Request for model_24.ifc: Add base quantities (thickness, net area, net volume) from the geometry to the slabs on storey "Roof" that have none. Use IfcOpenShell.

First a look at what the model holds.

```python
import ifcopenshell
import ifcopenshell.util.element
import ifcopenshell.util.unit

model = ifcopenshell.open("model_24.ifc")
print(model.schema)
for unit_type in ("LENGTHUNIT", "AREAUNIT", "VOLUMEUNIT"):
    print(unit_type, ifcopenshell.util.unit.calculate_unit_scale(model, unit_type))
storey = next(s for s in model.by_type("IfcBuildingStorey") if s.Name == "Roof")
slabs = [e for e in ifcopenshell.util.element.get_decomposition(storey) if e.is_a("IfcSlab")]
for e in sorted(slabs, key=lambda e: e.id()):
    print(e.id(), e.is_a(), e.Name, list(ifcopenshell.util.element.get_psets(e, qtos_only=True)), sep=" | ")
```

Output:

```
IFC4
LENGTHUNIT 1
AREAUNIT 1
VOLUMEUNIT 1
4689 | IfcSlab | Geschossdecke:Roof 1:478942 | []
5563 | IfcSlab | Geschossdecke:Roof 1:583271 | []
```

```python
import ifcopenshell
import ifcopenshell.api.pset
import ifcopenshell.geom
import ifcopenshell.util.element
import ifcopenshell.util.shape
import ifcopenshell.util.unit

model = ifcopenshell.open("model_24.ifc")
unit_scale = ifcopenshell.util.unit.calculate_unit_scale(model)
area_scale = ifcopenshell.util.unit.calculate_unit_scale(model, "AREAUNIT")
volume_scale = ifcopenshell.util.unit.calculate_unit_scale(model, "VOLUMEUNIT")
settings = ifcopenshell.geom.settings()

storey = next(s for s in model.by_type("IfcBuildingStorey") if s.Name == "Roof")
slabs = [e for e in ifcopenshell.util.element.get_decomposition(storey) if e.is_a("IfcSlab")]

for e in sorted(slabs, key=lambda e: e.id()):
    if ifcopenshell.util.element.get_psets(e, qtos_only=True, should_inherit=False):
        continue
    # Geometry comes back in metres, in the element's own axes.
    shape = ifcopenshell.geom.create_shape(settings, e)
    values = {
        "Width": ifcopenshell.util.shape.get_z(shape.geometry) / unit_scale,
        "NetArea": ifcopenshell.util.shape.get_footprint_area(shape.geometry) / area_scale,
        "NetVolume": ifcopenshell.util.shape.get_volume(shape.geometry) / volume_scale,
    }
    qto = ifcopenshell.api.pset.add_qto(model, product=e, name="Qto_SlabBaseQuantities")
    ifcopenshell.api.pset.edit_qto(model, qto=qto, properties=values)
    print(e.id(), {k: round(v, 3) for k, v in values.items()})

model.write("model_24-out.ifc")
```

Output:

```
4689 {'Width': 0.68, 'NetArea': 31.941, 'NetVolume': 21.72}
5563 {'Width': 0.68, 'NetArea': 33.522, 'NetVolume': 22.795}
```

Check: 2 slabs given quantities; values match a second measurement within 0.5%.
